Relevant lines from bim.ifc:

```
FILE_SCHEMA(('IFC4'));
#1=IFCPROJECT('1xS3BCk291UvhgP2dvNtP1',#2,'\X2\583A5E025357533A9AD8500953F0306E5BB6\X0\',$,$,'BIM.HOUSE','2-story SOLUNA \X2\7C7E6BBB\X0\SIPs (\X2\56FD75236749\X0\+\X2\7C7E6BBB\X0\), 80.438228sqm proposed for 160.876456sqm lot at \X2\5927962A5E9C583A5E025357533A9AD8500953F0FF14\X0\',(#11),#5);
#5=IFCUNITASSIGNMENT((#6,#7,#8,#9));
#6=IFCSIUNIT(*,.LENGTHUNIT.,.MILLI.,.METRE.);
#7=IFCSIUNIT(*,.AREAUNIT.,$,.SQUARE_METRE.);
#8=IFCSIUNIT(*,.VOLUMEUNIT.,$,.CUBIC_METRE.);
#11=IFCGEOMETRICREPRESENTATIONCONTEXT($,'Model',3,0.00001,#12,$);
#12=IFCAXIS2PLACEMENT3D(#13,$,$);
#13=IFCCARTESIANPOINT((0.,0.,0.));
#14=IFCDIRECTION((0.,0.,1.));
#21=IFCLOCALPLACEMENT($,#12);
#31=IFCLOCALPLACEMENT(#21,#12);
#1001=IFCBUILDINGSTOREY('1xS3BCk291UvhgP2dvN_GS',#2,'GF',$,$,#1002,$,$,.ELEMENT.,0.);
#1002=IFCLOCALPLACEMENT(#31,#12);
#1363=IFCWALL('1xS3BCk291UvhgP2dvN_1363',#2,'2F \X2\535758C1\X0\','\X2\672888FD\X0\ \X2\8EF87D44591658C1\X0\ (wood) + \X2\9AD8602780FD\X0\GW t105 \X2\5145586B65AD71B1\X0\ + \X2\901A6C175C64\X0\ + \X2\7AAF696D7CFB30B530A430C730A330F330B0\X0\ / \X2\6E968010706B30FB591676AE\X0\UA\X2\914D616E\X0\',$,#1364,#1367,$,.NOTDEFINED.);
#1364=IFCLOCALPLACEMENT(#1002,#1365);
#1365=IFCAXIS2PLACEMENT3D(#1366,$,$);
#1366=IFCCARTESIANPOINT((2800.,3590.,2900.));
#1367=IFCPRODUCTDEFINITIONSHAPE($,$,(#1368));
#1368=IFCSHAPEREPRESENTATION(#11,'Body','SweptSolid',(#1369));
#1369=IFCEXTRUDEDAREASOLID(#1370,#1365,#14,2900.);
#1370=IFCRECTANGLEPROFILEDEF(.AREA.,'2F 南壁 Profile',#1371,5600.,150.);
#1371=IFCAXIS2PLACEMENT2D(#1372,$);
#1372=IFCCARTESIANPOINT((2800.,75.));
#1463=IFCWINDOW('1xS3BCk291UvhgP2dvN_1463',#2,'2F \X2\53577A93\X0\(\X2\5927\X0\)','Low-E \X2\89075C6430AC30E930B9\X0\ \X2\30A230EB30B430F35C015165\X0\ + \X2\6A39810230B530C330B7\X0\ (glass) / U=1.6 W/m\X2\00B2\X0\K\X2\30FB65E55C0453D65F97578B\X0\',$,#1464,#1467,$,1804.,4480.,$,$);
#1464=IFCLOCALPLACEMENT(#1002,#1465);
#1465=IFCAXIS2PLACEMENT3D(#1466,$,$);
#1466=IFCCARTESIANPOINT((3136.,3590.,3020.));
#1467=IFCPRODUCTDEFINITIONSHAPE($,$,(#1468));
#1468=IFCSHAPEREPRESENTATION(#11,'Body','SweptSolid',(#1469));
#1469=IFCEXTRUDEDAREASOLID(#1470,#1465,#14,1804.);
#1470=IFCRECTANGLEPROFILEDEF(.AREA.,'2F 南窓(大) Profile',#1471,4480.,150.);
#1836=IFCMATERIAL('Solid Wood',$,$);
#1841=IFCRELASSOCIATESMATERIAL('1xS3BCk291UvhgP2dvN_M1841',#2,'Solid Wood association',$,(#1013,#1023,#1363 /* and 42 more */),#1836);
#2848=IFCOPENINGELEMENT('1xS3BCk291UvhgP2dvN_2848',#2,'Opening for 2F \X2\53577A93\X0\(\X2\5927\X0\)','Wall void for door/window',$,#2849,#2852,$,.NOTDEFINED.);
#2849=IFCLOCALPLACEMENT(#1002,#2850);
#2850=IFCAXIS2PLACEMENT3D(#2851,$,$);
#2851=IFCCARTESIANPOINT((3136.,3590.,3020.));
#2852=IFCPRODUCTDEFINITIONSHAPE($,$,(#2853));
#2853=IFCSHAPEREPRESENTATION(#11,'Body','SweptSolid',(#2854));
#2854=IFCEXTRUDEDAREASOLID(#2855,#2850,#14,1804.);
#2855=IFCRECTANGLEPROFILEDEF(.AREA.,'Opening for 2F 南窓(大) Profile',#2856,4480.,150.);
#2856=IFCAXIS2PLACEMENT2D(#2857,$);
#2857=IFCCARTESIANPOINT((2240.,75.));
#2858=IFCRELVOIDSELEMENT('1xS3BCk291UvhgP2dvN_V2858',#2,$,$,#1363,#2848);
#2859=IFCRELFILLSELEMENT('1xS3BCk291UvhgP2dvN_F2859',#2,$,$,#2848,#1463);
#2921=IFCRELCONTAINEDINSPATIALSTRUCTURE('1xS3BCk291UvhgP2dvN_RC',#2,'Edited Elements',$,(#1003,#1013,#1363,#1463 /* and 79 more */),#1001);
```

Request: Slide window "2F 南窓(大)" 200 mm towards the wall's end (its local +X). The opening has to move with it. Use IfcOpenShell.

```python
import ifcopenshell
import ifcopenshell.api.geometry
import ifcopenshell.util.placement

model = ifcopenshell.open("bim.ifc")

window = model.by_id(1463)
opening = window.FillsVoids[0].RelatingOpeningElement
wall = opening.VoidsElements[0].RelatingBuildingElement

wall_matrix = ifcopenshell.util.placement.get_local_placement(wall.ObjectPlacement)
shift = wall_matrix[:3, 0] * 200.0
before = ifcopenshell.util.placement.get_local_placement(window.ObjectPlacement)[:3, 3].copy()

# The window is not placed relative to its opening, so move both.
for product in (opening, window):
    matrix = ifcopenshell.util.placement.get_local_placement(product.ObjectPlacement)
    matrix[:3, 3] += shift
    ifcopenshell.api.geometry.edit_object_placement(model, product=product, matrix=matrix, is_si=False)

after = ifcopenshell.util.placement.get_local_placement(window.ObjectPlacement)[:3, 3]
print("window moved by", (after - before).round(3) + 0.0)

model.write("bim_rev.ifc")
```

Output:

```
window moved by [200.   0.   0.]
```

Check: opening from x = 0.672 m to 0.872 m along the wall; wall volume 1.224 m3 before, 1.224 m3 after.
